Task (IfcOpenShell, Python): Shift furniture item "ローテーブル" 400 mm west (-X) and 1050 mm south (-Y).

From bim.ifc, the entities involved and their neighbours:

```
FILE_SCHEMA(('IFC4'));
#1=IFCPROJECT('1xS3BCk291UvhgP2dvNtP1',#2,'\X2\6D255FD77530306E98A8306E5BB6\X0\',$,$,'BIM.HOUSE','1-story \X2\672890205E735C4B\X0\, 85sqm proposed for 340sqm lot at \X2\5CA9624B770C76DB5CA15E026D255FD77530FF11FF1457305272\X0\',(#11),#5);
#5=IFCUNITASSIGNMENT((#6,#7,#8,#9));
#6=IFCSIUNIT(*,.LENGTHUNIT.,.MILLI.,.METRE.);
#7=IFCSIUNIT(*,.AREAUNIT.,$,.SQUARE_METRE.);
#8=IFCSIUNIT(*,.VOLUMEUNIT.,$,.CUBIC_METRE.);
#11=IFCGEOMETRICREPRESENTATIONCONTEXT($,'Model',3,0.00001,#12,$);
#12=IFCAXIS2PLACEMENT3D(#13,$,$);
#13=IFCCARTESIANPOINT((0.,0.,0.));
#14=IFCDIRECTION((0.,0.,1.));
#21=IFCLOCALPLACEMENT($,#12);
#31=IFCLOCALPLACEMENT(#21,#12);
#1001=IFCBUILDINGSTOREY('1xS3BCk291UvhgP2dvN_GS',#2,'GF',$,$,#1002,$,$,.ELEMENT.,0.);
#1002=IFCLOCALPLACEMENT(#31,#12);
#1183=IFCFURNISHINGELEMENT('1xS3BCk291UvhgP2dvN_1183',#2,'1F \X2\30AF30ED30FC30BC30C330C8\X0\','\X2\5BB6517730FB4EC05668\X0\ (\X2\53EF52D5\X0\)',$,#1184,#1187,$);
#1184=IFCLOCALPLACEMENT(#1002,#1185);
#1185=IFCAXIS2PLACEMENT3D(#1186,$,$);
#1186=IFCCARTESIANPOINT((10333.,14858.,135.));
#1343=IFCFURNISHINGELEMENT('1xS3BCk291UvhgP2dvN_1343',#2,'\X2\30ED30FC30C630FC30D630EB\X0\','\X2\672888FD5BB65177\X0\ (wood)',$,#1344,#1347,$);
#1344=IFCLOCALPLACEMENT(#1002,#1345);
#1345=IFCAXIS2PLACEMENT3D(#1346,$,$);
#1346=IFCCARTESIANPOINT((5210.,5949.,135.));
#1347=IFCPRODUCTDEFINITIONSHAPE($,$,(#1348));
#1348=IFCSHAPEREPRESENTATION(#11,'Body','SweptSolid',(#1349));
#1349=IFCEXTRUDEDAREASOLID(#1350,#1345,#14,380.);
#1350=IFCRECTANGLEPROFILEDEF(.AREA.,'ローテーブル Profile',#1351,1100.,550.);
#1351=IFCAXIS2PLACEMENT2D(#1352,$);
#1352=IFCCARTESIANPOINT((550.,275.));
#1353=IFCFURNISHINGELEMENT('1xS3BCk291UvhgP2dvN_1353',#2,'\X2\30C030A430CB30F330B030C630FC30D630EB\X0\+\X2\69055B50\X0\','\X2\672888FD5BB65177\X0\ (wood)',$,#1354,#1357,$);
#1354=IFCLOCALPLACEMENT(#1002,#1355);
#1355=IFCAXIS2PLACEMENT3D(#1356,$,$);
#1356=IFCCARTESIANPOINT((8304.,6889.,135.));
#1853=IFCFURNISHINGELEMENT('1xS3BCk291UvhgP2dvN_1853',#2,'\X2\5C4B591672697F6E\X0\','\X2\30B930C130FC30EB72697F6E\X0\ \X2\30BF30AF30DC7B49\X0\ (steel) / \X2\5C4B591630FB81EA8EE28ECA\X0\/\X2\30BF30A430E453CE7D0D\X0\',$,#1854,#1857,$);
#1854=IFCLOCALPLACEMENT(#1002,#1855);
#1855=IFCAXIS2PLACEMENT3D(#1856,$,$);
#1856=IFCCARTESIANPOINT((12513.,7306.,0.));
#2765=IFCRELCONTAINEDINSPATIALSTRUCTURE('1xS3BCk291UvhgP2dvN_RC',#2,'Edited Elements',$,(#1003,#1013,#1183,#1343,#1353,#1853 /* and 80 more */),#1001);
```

```python
import ifcopenshell
import ifcopenshell.api.geometry
import ifcopenshell.util.placement
import ifcopenshell.util.unit

model = ifcopenshell.open("bim.ifc")
unit_scale = ifcopenshell.util.unit.calculate_unit_scale(model)

item = model.by_guid("1xS3BCk291UvhgP2dvN_1343")
matrix = ifcopenshell.util.placement.get_local_placement(item.ObjectPlacement)
matrix[0, 3] -= 0.4 / unit_scale
matrix[1, 3] -= 1.05 / unit_scale
ifcopenshell.api.geometry.edit_object_placement(model, product=item, matrix=matrix, is_si=False)

print(ifcopenshell.util.placement.get_local_placement(item.ObjectPlacement).round(3) + 0.0)

model.write("bim_v2.ifc")
```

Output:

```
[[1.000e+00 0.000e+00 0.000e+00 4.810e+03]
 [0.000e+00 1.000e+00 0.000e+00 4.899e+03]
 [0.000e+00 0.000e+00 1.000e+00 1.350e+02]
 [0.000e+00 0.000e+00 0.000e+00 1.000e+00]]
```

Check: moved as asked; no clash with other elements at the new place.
